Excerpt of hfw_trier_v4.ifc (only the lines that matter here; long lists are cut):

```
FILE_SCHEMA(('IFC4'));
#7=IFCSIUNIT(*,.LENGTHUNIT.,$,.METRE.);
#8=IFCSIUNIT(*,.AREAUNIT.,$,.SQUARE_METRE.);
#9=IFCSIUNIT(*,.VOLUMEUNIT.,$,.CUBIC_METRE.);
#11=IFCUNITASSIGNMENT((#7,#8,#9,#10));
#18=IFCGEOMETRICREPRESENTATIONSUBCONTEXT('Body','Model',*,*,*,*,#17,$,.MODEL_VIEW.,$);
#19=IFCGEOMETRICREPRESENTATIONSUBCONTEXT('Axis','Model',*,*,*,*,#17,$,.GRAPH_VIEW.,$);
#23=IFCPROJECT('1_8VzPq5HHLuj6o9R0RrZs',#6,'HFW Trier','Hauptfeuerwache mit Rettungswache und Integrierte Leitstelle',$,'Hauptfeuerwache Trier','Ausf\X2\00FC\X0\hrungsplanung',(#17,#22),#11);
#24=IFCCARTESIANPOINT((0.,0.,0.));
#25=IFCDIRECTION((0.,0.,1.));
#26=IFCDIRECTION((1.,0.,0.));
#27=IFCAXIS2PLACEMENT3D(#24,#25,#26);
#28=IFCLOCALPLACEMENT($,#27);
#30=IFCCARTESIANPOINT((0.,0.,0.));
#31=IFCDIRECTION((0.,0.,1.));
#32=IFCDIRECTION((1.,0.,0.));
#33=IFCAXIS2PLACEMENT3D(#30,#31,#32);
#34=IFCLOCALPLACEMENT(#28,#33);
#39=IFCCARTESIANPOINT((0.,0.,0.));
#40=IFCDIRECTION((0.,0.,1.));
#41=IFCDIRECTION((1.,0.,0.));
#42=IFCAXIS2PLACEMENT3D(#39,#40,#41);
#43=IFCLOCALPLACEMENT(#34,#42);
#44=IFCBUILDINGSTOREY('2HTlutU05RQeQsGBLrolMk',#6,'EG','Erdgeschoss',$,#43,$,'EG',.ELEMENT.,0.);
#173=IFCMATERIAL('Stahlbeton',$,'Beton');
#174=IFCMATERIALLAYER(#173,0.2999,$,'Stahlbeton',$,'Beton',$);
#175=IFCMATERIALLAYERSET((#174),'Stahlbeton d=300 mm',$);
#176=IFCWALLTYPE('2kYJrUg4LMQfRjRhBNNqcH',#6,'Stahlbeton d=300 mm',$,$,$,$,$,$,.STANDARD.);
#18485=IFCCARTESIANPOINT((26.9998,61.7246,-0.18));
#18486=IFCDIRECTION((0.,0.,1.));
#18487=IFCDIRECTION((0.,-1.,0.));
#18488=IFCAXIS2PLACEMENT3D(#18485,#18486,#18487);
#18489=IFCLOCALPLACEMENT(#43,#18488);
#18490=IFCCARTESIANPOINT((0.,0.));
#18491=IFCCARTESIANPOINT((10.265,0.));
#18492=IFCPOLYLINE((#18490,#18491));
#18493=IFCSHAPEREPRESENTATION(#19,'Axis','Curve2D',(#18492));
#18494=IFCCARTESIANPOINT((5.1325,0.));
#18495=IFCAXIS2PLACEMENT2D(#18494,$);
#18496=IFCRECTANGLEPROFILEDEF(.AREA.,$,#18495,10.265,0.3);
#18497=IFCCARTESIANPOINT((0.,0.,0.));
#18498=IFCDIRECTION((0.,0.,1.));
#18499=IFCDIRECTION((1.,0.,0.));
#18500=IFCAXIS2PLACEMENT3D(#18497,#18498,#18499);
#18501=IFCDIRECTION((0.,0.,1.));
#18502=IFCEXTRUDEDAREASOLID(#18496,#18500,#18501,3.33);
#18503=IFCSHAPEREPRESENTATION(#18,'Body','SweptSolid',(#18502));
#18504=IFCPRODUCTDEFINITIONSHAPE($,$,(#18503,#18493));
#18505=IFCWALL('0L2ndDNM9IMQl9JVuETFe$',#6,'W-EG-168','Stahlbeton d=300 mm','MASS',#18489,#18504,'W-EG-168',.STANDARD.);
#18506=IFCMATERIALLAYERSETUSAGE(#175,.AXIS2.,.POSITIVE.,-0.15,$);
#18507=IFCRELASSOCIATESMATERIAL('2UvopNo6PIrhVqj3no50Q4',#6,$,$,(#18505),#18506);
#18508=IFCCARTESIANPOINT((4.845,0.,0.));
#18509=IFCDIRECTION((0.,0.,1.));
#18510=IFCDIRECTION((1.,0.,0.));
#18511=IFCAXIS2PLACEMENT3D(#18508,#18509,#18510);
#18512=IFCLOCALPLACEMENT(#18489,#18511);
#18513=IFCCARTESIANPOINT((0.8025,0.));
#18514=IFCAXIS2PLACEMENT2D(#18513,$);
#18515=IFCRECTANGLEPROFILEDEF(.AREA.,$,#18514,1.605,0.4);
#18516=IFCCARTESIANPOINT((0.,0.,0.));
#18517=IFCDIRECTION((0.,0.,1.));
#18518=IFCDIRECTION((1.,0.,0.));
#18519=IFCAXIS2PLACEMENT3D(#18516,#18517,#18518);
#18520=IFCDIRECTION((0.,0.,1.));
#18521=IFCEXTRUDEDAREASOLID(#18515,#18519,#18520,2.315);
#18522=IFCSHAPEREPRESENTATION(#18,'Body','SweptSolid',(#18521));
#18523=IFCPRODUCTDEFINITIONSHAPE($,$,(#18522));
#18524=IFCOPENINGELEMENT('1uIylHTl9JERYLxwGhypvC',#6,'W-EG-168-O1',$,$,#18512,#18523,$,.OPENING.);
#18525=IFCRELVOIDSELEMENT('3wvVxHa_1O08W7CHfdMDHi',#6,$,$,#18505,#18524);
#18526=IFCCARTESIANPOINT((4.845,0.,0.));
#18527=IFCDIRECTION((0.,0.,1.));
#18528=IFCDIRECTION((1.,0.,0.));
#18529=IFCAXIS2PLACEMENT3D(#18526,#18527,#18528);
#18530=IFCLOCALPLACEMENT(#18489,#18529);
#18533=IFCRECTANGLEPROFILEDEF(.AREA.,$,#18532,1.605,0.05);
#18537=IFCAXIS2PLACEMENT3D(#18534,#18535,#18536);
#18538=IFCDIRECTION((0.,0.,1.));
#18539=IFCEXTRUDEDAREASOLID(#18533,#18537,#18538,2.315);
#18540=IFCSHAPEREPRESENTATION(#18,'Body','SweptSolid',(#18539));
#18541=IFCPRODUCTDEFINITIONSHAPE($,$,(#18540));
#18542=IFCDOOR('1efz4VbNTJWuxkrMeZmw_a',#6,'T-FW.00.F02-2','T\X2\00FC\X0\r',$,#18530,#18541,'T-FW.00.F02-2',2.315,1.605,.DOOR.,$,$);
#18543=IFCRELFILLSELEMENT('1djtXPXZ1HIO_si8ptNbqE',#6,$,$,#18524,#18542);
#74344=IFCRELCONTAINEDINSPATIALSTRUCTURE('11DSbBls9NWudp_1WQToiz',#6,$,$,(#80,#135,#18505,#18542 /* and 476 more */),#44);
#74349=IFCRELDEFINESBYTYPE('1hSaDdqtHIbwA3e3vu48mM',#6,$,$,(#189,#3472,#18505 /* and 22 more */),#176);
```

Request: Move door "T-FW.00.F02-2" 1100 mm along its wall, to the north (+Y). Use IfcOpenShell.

```python
import ifcopenshell
import ifcopenshell.api.geometry
import ifcopenshell.util.placement
import ifcopenshell.util.unit

model = ifcopenshell.open("hfw_trier_v4.ifc")
unit_scale = ifcopenshell.util.unit.calculate_unit_scale(model)

door = model.by_guid("1efz4VbNTJWuxkrMeZmw_a")
opening = door.FillsVoids[0].RelatingOpeningElement
wall = opening.VoidsElements[0].RelatingBuildingElement

wall_matrix = ifcopenshell.util.placement.get_local_placement(wall.ObjectPlacement)
shift = wall_matrix[:3, 0] * -1.1 / unit_scale
before = ifcopenshell.util.placement.get_local_placement(door.ObjectPlacement)[:3, 3].copy()

# The door is not placed relative to its opening, so move both.
for product in (opening, door):
    matrix = ifcopenshell.util.placement.get_local_placement(product.ObjectPlacement)
    matrix[:3, 3] += shift
    ifcopenshell.api.geometry.edit_object_placement(model, product=product, matrix=matrix, is_si=False)

after = ifcopenshell.util.placement.get_local_placement(door.ObjectPlacement)[:3, 3]
print("door moved by", (after - before).round(3) + 0.0)

model.write("hfw_trier_v4_v2.ifc")
```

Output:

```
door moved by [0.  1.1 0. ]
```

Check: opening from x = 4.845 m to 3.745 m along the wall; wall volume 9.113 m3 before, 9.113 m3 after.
